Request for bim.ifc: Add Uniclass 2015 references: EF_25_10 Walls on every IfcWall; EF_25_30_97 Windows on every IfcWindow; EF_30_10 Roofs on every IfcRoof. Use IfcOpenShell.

First a look at what the model holds.

```python
import ifcopenshell

model = ifcopenshell.open("bim.ifc")
print(model.schema)
print("classifications:", [c.Name for c in model.by_type("IfcClassification")])
for ifc_class in ("IfcDoor", "IfcRoof", "IfcStair", "IfcWall", "IfcWindow"):
    print(ifc_class, len(model.by_type(ifc_class)))
```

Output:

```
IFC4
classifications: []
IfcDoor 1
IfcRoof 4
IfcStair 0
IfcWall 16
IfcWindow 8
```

```python
import ifcopenshell
import ifcopenshell.api.classification

model = ifcopenshell.open("bim.ifc")

system = ifcopenshell.api.classification.add_classification(model, classification="Uniclass 2015")

codes = {
    "IfcWall": ("EF_25_10", "Walls"),
    "IfcWindow": ("EF_25_30_97", "Windows"),
    "IfcRoof": ("EF_30_10", "Roofs"),
}
for ifc_class, (code, name) in codes.items():
    products = model.by_type(ifc_class)
    ifcopenshell.api.classification.add_reference(
        model, products=products, classification=system, identification=code, name=name
    )
    print(code, len(products))

model.write("bim_rev.ifc")
```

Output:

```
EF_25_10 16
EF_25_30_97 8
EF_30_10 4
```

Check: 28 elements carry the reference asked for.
